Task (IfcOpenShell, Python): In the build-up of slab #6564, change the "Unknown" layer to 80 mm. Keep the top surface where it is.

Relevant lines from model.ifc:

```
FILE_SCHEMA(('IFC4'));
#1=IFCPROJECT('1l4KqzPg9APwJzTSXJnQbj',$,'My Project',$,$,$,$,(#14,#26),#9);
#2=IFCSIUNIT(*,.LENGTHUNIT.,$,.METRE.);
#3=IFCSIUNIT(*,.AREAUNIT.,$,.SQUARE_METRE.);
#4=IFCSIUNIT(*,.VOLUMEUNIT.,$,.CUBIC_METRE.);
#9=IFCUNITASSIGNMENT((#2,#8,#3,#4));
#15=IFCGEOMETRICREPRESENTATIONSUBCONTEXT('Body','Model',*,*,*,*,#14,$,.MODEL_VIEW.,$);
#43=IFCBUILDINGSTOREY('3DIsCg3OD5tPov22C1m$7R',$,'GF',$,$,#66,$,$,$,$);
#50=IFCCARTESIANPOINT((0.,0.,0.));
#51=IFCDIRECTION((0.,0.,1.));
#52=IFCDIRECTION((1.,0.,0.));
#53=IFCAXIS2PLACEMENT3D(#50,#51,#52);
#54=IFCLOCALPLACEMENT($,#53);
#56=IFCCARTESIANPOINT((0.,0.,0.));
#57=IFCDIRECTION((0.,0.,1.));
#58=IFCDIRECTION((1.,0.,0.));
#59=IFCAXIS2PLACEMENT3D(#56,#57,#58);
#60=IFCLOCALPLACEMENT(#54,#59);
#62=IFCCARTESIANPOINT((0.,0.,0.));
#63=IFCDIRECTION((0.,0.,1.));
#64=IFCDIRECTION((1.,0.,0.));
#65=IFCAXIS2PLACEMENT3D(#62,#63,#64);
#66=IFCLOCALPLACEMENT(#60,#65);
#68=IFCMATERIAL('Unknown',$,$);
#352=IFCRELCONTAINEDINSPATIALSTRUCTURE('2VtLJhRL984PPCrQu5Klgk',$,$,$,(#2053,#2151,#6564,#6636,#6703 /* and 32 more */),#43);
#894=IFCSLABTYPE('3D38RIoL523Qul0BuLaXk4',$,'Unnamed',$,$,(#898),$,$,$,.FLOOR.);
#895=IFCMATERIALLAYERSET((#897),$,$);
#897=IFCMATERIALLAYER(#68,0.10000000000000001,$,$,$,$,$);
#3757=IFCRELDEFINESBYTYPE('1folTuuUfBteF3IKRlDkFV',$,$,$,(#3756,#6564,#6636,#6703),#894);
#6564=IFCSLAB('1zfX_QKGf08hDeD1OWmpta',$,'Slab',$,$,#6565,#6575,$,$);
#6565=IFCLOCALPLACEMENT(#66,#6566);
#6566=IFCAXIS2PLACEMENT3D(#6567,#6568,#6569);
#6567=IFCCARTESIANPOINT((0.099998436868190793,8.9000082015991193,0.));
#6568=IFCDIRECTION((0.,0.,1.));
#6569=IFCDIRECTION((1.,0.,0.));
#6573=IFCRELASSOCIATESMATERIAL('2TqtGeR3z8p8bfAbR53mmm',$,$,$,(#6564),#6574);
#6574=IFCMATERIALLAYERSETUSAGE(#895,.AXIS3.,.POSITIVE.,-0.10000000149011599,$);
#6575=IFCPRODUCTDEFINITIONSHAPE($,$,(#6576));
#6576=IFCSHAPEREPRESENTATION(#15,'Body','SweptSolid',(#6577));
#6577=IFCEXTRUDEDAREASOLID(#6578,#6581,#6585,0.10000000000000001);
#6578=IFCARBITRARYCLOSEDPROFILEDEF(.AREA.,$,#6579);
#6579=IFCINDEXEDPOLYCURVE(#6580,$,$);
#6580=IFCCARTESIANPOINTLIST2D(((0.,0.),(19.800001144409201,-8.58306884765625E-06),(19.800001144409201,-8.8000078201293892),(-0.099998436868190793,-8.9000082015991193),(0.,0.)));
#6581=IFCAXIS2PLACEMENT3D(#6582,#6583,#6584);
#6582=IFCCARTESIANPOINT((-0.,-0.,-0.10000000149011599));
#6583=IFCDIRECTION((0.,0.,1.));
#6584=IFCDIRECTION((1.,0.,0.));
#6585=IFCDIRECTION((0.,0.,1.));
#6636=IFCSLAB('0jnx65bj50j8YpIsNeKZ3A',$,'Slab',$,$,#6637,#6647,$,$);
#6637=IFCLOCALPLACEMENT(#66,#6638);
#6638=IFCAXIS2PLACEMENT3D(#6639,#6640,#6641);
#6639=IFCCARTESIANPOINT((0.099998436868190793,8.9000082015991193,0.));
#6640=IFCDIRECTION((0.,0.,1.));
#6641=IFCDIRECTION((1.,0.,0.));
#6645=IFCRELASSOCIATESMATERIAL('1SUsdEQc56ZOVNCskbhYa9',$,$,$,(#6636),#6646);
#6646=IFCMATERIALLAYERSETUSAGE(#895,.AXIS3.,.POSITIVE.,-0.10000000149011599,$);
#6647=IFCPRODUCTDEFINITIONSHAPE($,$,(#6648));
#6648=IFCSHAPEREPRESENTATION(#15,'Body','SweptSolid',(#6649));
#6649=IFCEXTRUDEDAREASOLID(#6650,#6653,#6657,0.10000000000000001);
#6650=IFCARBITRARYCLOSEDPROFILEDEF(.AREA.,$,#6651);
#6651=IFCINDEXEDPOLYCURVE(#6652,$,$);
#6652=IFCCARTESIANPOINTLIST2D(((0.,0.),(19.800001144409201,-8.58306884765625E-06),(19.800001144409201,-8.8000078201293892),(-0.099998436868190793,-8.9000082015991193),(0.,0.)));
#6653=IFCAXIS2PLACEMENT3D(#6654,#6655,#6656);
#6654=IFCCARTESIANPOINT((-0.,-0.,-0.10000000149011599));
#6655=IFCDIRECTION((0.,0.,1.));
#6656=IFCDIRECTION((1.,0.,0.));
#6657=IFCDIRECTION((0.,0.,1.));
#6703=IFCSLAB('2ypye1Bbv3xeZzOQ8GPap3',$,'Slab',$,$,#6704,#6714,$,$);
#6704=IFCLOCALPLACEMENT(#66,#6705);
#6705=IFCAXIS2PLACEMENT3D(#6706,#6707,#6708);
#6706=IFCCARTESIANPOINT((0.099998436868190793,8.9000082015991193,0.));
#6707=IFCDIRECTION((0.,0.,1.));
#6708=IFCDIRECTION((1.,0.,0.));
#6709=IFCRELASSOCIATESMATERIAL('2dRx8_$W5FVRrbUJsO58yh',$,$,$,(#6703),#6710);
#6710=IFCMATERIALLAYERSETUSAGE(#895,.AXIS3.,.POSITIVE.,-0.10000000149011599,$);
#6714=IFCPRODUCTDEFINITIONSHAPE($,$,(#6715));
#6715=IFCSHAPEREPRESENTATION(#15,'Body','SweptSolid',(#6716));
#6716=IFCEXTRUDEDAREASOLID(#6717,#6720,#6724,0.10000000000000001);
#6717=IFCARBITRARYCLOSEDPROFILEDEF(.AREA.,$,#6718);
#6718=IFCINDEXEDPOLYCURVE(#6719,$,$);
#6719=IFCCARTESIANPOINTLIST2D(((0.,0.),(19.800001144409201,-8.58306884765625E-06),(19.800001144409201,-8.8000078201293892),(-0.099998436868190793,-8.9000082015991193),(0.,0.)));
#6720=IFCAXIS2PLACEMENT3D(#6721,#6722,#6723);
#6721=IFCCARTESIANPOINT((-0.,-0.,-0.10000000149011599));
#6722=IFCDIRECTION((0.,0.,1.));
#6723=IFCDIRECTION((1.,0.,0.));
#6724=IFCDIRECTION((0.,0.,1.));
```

```python
import ifcopenshell
import ifcopenshell.util.element
import ifcopenshell.util.representation
import ifcopenshell.util.unit

model = ifcopenshell.open("model.ifc")
unit_scale = ifcopenshell.util.unit.calculate_unit_scale(model)

layer_set = model.by_id(895)
layer = next(l for l in layer_set.MaterialLayers if l.Material and l.Material.Name == "Unknown")
change = 0.08 / unit_scale - layer.LayerThickness
layer.LayerThickness += change

# The layer set is shared, so every slab that uses it gets the new thickness.
slabs = [e for e in ifcopenshell.util.element.get_elements_by_material(model, layer_set) if e.is_a("IfcSlab")]
for slab in sorted(slabs, key=lambda e: e.id()):
    body = ifcopenshell.util.representation.get_representation(slab, "Model", "Body")
    solid = body.Items[0]
    old_depth = solid.Depth
    solid.Depth += change
    # Extruded upwards: lower the start of the extrusion so the top stays.
    x, y, z = solid.Position.Location.Coordinates
    solid.Position.Location = model.createIfcCartesianPoint((x, y, z - change))
    print(slab.id(), f"{old_depth:g} -> {solid.Depth:g}")

# The layers are counted up from the underside, which has moved.
for usage in {ifcopenshell.util.element.get_material(slab) for slab in slabs}:
    usage.OffsetFromReferenceLine -= change

model.write("model_edited.ifc")
```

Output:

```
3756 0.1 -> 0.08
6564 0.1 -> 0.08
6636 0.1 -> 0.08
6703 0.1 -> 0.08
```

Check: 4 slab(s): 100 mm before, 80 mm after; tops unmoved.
